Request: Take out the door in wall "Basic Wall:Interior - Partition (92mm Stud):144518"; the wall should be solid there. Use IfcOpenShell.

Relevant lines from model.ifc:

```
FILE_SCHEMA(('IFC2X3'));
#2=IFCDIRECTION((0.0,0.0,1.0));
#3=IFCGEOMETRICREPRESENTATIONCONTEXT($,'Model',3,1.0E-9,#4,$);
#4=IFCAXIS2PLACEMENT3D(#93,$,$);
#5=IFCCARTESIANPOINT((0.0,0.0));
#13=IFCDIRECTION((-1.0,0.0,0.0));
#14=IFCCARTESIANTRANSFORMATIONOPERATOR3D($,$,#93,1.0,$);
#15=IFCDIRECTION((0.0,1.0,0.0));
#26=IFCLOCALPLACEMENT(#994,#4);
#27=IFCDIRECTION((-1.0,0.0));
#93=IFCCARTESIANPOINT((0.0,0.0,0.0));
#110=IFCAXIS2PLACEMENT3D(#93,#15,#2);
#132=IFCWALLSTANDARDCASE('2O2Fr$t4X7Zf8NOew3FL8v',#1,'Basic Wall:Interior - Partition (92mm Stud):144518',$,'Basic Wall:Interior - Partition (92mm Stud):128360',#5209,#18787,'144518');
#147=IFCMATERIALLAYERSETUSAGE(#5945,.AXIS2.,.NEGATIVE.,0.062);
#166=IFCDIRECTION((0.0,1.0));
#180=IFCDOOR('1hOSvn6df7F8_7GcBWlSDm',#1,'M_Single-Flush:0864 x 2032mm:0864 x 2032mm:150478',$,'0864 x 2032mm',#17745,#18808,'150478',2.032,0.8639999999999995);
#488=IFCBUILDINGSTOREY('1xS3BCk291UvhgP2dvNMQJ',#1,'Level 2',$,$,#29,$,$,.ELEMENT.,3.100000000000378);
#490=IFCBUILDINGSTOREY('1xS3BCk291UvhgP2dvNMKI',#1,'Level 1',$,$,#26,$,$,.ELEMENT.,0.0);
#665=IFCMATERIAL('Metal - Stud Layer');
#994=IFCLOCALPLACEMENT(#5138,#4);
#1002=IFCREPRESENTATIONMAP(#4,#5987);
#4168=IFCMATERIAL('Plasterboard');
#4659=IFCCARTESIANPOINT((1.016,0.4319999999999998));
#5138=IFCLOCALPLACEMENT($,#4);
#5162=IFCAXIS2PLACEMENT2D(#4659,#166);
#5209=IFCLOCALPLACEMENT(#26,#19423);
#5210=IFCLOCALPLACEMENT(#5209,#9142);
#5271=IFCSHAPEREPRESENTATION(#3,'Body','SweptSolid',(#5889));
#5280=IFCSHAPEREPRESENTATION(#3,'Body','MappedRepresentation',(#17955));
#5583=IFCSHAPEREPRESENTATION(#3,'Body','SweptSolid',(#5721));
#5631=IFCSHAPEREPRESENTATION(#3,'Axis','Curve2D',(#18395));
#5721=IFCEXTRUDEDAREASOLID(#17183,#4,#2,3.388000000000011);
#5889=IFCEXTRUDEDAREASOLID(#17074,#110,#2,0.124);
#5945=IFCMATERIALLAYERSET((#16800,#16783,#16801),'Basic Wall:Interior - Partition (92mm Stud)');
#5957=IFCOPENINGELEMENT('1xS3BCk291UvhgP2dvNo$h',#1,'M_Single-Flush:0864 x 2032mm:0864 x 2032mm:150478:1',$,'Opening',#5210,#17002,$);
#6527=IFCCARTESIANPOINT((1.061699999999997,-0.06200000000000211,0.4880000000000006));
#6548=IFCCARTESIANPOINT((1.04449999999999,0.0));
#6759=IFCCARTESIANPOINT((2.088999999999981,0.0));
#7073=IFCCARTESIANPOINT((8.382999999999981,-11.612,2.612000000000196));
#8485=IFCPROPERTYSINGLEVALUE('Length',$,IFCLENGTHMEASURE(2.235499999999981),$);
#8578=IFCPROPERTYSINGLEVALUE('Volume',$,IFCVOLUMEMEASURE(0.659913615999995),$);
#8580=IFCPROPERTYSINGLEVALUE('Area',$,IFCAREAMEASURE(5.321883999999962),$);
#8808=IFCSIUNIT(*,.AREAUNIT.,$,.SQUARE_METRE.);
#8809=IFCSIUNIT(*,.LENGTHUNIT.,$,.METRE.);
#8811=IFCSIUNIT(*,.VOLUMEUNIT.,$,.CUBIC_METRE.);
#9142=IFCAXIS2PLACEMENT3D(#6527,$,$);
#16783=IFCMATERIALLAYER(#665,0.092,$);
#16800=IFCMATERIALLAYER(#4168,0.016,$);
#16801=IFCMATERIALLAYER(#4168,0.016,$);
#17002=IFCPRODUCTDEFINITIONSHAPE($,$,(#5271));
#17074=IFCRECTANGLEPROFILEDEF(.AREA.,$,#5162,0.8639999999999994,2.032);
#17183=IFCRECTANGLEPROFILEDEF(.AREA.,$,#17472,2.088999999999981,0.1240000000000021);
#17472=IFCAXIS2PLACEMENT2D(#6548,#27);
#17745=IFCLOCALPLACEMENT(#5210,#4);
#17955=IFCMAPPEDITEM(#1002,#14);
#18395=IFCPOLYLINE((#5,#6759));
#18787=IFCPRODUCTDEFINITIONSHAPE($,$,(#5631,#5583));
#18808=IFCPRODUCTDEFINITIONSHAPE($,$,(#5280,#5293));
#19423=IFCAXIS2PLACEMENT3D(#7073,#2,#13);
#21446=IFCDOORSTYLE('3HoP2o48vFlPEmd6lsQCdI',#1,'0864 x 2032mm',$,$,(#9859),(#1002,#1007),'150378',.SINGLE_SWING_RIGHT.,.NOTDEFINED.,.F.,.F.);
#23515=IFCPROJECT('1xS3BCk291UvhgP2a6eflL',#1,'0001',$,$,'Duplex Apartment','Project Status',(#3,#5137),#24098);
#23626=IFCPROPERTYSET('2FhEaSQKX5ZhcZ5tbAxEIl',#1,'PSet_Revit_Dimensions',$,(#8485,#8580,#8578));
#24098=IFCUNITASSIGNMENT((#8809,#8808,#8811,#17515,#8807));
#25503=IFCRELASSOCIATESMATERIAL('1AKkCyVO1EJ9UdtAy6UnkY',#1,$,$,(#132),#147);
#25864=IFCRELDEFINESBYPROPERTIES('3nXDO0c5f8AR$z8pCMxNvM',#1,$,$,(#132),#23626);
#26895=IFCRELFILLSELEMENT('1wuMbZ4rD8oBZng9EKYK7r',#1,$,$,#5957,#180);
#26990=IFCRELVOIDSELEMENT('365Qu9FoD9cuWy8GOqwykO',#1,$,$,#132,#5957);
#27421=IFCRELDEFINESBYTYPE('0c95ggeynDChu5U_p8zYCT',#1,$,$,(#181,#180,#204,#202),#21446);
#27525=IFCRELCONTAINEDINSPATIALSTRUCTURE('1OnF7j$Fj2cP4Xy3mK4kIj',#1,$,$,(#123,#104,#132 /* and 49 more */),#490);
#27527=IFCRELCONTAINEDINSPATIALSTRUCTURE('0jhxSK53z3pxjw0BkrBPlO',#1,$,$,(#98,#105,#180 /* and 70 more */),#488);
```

```python
import ifcopenshell
import ifcopenshell.api.feature
import ifcopenshell.api.pset
import ifcopenshell.api.root
import ifcopenshell.geom
import ifcopenshell.util.element
import ifcopenshell.util.shape
import ifcopenshell.util.unit

model = ifcopenshell.open("model.ifc")
area_scale = ifcopenshell.util.unit.calculate_unit_scale(model, "AREAUNIT")
volume_scale = ifcopenshell.util.unit.calculate_unit_scale(model, "VOLUMEUNIT")
settings = ifcopenshell.geom.settings()


def volume(element):
    """Net volume in cubic metres, openings subtracted."""
    shape = ifcopenshell.geom.create_shape(settings, element)
    return ifcopenshell.util.shape.get_volume(shape.geometry)


door = model.by_guid("1hOSvn6df7F8_7GcBWlSDm")
opening = door.FillsVoids[0].RelatingOpeningElement
wall = opening.VoidsElements[0].RelatingBuildingElement
before = volume(wall)

ifcopenshell.api.root.remove_product(model, product=door)
ifcopenshell.api.feature.remove_feature(model, feature=opening)

after = volume(wall)
thickness = 0.124  # wall thickness in metres

# Update the wall's stored quantities.
pset = model.by_id(ifcopenshell.util.element.get_pset(wall, "PSet_Revit_Dimensions", should_inherit=False)["id"])
ifcopenshell.api.pset.edit_pset(model, pset=pset, properties={
    "Area": model.create_entity("IfcAreaMeasure", after / thickness / area_scale),
    "Volume": model.create_entity("IfcVolumeMeasure", after / volume_scale),
})

print(f"wall volume {before:.3f} -> {after:.3f} m3")

model.write("model_updated.ifc")
```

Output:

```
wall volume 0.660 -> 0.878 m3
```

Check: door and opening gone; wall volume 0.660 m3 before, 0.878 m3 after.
